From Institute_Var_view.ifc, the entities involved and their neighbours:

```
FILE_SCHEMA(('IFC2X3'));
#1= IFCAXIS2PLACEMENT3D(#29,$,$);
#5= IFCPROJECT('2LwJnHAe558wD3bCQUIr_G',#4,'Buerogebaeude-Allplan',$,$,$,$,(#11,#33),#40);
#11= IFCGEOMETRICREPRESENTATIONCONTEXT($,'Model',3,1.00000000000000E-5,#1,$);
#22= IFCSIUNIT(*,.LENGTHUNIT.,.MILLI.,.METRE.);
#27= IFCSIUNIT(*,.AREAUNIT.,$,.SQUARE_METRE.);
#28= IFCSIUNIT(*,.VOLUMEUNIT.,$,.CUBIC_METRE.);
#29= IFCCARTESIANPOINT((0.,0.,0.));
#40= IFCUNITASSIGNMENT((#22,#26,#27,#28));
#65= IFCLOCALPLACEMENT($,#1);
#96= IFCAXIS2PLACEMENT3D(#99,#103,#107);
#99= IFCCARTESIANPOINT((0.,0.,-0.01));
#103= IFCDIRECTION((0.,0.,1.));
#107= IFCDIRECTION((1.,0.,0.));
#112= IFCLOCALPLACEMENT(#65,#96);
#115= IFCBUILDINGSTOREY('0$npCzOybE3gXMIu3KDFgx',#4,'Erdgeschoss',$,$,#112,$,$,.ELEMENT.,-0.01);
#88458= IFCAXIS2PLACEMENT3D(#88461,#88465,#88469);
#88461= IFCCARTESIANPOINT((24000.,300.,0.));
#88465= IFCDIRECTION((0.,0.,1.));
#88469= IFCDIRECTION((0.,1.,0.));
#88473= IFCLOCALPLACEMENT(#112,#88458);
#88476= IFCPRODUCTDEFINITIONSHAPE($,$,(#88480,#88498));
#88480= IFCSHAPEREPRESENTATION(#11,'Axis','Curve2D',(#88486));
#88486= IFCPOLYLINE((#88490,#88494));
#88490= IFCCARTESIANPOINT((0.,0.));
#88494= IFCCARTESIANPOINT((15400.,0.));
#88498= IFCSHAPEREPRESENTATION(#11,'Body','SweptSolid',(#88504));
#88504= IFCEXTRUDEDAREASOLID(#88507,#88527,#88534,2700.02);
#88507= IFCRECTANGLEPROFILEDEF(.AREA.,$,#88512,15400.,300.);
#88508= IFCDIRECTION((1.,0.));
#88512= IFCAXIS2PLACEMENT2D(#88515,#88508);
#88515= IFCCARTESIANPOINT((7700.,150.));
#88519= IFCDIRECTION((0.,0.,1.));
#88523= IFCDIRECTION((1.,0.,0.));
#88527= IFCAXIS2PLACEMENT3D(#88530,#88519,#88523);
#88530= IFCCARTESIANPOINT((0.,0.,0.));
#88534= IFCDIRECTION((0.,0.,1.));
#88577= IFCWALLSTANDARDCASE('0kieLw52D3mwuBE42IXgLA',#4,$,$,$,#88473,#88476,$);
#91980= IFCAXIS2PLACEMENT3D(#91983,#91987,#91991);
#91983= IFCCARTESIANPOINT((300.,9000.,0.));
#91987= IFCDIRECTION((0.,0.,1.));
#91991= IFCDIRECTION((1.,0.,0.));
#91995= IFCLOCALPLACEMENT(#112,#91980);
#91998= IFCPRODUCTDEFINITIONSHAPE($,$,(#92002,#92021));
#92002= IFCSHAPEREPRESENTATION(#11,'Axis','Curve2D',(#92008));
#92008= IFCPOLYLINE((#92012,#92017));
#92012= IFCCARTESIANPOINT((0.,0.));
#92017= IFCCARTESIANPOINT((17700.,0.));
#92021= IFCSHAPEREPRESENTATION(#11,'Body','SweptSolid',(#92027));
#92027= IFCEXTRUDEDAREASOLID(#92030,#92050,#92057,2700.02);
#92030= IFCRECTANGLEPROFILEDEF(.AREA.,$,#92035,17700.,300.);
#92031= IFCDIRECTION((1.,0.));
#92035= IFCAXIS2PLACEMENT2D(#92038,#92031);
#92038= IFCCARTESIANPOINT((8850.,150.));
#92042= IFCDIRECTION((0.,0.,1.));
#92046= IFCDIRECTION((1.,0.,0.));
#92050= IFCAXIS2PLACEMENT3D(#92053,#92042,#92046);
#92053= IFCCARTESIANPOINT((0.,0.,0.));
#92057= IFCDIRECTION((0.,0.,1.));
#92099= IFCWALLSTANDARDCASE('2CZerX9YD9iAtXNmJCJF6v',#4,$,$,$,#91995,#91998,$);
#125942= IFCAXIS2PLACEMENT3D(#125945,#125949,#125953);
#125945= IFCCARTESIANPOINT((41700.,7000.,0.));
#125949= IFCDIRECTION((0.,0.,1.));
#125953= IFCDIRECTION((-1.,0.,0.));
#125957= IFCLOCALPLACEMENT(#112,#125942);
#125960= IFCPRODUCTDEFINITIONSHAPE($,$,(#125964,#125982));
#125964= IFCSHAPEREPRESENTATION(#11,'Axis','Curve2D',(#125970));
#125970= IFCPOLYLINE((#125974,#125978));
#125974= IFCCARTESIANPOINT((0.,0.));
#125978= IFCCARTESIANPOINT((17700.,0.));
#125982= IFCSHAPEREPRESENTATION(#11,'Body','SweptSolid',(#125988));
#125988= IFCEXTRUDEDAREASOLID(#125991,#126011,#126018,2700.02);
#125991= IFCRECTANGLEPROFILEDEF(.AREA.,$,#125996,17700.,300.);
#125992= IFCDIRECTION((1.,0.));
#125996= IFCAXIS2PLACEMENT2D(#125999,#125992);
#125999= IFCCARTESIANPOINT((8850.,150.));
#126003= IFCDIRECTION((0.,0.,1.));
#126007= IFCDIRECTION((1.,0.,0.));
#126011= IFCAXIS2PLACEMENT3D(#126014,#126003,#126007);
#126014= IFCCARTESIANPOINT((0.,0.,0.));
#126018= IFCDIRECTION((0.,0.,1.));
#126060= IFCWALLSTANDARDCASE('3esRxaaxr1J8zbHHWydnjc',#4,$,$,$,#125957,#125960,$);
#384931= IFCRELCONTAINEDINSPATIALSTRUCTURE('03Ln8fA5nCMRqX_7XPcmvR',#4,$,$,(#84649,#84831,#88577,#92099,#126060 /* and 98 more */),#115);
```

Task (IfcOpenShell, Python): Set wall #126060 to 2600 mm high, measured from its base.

```python
import ifcopenshell
import ifcopenshell.geom
import ifcopenshell.util.shape
import ifcopenshell.util.unit

model = ifcopenshell.open("Institute_Var_view.ifc")
unit_scale = ifcopenshell.util.unit.calculate_unit_scale(model)
settings = ifcopenshell.geom.settings()


def volume(element):
    """Net volume in cubic metres, openings subtracted."""
    shape = ifcopenshell.geom.create_shape(settings, element)
    return ifcopenshell.util.shape.get_volume(shape.geometry)


wall = model.by_guid("3esRxaaxr1J8zbHHWydnjc")
before = volume(wall)

body = next(r for r in wall.Representation.Representations if r.RepresentationIdentifier == "Body")
solid = body.Items[0]
old_height = solid.Depth
solid.Depth = 2.6 / unit_scale
after = volume(wall)

print(f"height {old_height:g} -> {solid.Depth:g}, volume {before:.3f} -> {after:.3f} m3")

model.write("Institute_Var_view_updated.ifc")
```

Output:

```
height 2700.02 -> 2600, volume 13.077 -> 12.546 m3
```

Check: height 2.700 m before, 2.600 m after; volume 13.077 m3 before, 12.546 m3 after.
